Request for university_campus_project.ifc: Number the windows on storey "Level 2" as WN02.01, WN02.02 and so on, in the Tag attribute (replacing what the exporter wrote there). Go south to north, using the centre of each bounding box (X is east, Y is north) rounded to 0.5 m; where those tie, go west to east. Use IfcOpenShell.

First a look at what the model holds.

```python
import ifcopenshell
import ifcopenshell.util.element
import ifcopenshell.util.placement

model = ifcopenshell.open("university_campus_project.ifc")
print(model.schema)
storey = next(s for s in model.by_type("IfcBuildingStorey") if s.Name == "Level 2")
windows = [e for e in ifcopenshell.util.element.get_decomposition(storey) if e.is_a("IfcWindow")]
for e in sorted(windows, key=lambda e: e.id()):
    origin = ifcopenshell.util.placement.get_local_placement(e.ObjectPlacement)[:3, 3]
    print(e.id(), e.Tag, e.Name, origin.round(2) + 0.0, sep=" | ")
```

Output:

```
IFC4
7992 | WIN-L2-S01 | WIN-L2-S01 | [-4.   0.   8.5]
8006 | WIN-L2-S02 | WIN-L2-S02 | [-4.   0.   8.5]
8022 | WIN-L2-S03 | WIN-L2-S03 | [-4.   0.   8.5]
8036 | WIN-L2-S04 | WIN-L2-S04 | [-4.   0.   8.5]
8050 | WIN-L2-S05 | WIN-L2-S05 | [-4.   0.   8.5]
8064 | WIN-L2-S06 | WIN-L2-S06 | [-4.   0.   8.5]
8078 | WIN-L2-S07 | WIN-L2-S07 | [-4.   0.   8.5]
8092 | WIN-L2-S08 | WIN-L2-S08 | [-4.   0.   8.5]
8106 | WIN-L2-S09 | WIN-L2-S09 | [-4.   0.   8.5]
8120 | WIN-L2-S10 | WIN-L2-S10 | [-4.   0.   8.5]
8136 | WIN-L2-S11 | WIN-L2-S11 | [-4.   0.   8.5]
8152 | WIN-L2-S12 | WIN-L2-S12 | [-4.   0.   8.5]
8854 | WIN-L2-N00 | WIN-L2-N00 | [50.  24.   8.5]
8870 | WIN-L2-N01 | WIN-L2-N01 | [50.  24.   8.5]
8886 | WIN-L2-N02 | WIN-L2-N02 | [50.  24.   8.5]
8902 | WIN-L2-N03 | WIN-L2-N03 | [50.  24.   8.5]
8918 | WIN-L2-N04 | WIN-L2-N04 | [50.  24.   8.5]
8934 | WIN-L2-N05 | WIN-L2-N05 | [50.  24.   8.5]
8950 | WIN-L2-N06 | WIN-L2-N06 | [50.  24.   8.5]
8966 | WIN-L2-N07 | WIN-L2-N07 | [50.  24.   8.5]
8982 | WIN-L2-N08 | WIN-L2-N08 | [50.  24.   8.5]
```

```python
import ifcopenshell
import ifcopenshell.geom
import ifcopenshell.util.element
import ifcopenshell.util.shape

model = ifcopenshell.open("university_campus_project.ifc")
settings = ifcopenshell.geom.settings()
settings.set("use-world-coords", True)


def centre(element):
    shape = ifcopenshell.geom.create_shape(settings, element)
    return ifcopenshell.util.shape.get_bbox_centroid(shape.geometry)


storey = next(s for s in model.by_type("IfcBuildingStorey") if s.Name == "Level 2")
windows = [e for e in ifcopenshell.util.element.get_decomposition(storey) if e.is_a("IfcWindow")]

# Insertion points can sit at a corner or the storey origin, so sort by the geometry (in metres).
centres = {e: centre(e) for e in windows}
windows.sort(key=lambda e: (round(centres[e][1] / 0.5), centres[e][0]))

for i, e in enumerate(windows, start=1):
    number = f"WN02.{i:02d}"
    e.Tag = number
    print(e.id(), number)

model.write("university_campus_project-out.ifc")
```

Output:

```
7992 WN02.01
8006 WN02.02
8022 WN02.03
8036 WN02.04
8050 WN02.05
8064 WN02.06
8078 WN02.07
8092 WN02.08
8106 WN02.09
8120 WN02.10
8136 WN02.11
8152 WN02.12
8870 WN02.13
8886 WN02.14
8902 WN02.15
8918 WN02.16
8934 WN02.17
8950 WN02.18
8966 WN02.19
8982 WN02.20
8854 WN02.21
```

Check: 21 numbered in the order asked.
